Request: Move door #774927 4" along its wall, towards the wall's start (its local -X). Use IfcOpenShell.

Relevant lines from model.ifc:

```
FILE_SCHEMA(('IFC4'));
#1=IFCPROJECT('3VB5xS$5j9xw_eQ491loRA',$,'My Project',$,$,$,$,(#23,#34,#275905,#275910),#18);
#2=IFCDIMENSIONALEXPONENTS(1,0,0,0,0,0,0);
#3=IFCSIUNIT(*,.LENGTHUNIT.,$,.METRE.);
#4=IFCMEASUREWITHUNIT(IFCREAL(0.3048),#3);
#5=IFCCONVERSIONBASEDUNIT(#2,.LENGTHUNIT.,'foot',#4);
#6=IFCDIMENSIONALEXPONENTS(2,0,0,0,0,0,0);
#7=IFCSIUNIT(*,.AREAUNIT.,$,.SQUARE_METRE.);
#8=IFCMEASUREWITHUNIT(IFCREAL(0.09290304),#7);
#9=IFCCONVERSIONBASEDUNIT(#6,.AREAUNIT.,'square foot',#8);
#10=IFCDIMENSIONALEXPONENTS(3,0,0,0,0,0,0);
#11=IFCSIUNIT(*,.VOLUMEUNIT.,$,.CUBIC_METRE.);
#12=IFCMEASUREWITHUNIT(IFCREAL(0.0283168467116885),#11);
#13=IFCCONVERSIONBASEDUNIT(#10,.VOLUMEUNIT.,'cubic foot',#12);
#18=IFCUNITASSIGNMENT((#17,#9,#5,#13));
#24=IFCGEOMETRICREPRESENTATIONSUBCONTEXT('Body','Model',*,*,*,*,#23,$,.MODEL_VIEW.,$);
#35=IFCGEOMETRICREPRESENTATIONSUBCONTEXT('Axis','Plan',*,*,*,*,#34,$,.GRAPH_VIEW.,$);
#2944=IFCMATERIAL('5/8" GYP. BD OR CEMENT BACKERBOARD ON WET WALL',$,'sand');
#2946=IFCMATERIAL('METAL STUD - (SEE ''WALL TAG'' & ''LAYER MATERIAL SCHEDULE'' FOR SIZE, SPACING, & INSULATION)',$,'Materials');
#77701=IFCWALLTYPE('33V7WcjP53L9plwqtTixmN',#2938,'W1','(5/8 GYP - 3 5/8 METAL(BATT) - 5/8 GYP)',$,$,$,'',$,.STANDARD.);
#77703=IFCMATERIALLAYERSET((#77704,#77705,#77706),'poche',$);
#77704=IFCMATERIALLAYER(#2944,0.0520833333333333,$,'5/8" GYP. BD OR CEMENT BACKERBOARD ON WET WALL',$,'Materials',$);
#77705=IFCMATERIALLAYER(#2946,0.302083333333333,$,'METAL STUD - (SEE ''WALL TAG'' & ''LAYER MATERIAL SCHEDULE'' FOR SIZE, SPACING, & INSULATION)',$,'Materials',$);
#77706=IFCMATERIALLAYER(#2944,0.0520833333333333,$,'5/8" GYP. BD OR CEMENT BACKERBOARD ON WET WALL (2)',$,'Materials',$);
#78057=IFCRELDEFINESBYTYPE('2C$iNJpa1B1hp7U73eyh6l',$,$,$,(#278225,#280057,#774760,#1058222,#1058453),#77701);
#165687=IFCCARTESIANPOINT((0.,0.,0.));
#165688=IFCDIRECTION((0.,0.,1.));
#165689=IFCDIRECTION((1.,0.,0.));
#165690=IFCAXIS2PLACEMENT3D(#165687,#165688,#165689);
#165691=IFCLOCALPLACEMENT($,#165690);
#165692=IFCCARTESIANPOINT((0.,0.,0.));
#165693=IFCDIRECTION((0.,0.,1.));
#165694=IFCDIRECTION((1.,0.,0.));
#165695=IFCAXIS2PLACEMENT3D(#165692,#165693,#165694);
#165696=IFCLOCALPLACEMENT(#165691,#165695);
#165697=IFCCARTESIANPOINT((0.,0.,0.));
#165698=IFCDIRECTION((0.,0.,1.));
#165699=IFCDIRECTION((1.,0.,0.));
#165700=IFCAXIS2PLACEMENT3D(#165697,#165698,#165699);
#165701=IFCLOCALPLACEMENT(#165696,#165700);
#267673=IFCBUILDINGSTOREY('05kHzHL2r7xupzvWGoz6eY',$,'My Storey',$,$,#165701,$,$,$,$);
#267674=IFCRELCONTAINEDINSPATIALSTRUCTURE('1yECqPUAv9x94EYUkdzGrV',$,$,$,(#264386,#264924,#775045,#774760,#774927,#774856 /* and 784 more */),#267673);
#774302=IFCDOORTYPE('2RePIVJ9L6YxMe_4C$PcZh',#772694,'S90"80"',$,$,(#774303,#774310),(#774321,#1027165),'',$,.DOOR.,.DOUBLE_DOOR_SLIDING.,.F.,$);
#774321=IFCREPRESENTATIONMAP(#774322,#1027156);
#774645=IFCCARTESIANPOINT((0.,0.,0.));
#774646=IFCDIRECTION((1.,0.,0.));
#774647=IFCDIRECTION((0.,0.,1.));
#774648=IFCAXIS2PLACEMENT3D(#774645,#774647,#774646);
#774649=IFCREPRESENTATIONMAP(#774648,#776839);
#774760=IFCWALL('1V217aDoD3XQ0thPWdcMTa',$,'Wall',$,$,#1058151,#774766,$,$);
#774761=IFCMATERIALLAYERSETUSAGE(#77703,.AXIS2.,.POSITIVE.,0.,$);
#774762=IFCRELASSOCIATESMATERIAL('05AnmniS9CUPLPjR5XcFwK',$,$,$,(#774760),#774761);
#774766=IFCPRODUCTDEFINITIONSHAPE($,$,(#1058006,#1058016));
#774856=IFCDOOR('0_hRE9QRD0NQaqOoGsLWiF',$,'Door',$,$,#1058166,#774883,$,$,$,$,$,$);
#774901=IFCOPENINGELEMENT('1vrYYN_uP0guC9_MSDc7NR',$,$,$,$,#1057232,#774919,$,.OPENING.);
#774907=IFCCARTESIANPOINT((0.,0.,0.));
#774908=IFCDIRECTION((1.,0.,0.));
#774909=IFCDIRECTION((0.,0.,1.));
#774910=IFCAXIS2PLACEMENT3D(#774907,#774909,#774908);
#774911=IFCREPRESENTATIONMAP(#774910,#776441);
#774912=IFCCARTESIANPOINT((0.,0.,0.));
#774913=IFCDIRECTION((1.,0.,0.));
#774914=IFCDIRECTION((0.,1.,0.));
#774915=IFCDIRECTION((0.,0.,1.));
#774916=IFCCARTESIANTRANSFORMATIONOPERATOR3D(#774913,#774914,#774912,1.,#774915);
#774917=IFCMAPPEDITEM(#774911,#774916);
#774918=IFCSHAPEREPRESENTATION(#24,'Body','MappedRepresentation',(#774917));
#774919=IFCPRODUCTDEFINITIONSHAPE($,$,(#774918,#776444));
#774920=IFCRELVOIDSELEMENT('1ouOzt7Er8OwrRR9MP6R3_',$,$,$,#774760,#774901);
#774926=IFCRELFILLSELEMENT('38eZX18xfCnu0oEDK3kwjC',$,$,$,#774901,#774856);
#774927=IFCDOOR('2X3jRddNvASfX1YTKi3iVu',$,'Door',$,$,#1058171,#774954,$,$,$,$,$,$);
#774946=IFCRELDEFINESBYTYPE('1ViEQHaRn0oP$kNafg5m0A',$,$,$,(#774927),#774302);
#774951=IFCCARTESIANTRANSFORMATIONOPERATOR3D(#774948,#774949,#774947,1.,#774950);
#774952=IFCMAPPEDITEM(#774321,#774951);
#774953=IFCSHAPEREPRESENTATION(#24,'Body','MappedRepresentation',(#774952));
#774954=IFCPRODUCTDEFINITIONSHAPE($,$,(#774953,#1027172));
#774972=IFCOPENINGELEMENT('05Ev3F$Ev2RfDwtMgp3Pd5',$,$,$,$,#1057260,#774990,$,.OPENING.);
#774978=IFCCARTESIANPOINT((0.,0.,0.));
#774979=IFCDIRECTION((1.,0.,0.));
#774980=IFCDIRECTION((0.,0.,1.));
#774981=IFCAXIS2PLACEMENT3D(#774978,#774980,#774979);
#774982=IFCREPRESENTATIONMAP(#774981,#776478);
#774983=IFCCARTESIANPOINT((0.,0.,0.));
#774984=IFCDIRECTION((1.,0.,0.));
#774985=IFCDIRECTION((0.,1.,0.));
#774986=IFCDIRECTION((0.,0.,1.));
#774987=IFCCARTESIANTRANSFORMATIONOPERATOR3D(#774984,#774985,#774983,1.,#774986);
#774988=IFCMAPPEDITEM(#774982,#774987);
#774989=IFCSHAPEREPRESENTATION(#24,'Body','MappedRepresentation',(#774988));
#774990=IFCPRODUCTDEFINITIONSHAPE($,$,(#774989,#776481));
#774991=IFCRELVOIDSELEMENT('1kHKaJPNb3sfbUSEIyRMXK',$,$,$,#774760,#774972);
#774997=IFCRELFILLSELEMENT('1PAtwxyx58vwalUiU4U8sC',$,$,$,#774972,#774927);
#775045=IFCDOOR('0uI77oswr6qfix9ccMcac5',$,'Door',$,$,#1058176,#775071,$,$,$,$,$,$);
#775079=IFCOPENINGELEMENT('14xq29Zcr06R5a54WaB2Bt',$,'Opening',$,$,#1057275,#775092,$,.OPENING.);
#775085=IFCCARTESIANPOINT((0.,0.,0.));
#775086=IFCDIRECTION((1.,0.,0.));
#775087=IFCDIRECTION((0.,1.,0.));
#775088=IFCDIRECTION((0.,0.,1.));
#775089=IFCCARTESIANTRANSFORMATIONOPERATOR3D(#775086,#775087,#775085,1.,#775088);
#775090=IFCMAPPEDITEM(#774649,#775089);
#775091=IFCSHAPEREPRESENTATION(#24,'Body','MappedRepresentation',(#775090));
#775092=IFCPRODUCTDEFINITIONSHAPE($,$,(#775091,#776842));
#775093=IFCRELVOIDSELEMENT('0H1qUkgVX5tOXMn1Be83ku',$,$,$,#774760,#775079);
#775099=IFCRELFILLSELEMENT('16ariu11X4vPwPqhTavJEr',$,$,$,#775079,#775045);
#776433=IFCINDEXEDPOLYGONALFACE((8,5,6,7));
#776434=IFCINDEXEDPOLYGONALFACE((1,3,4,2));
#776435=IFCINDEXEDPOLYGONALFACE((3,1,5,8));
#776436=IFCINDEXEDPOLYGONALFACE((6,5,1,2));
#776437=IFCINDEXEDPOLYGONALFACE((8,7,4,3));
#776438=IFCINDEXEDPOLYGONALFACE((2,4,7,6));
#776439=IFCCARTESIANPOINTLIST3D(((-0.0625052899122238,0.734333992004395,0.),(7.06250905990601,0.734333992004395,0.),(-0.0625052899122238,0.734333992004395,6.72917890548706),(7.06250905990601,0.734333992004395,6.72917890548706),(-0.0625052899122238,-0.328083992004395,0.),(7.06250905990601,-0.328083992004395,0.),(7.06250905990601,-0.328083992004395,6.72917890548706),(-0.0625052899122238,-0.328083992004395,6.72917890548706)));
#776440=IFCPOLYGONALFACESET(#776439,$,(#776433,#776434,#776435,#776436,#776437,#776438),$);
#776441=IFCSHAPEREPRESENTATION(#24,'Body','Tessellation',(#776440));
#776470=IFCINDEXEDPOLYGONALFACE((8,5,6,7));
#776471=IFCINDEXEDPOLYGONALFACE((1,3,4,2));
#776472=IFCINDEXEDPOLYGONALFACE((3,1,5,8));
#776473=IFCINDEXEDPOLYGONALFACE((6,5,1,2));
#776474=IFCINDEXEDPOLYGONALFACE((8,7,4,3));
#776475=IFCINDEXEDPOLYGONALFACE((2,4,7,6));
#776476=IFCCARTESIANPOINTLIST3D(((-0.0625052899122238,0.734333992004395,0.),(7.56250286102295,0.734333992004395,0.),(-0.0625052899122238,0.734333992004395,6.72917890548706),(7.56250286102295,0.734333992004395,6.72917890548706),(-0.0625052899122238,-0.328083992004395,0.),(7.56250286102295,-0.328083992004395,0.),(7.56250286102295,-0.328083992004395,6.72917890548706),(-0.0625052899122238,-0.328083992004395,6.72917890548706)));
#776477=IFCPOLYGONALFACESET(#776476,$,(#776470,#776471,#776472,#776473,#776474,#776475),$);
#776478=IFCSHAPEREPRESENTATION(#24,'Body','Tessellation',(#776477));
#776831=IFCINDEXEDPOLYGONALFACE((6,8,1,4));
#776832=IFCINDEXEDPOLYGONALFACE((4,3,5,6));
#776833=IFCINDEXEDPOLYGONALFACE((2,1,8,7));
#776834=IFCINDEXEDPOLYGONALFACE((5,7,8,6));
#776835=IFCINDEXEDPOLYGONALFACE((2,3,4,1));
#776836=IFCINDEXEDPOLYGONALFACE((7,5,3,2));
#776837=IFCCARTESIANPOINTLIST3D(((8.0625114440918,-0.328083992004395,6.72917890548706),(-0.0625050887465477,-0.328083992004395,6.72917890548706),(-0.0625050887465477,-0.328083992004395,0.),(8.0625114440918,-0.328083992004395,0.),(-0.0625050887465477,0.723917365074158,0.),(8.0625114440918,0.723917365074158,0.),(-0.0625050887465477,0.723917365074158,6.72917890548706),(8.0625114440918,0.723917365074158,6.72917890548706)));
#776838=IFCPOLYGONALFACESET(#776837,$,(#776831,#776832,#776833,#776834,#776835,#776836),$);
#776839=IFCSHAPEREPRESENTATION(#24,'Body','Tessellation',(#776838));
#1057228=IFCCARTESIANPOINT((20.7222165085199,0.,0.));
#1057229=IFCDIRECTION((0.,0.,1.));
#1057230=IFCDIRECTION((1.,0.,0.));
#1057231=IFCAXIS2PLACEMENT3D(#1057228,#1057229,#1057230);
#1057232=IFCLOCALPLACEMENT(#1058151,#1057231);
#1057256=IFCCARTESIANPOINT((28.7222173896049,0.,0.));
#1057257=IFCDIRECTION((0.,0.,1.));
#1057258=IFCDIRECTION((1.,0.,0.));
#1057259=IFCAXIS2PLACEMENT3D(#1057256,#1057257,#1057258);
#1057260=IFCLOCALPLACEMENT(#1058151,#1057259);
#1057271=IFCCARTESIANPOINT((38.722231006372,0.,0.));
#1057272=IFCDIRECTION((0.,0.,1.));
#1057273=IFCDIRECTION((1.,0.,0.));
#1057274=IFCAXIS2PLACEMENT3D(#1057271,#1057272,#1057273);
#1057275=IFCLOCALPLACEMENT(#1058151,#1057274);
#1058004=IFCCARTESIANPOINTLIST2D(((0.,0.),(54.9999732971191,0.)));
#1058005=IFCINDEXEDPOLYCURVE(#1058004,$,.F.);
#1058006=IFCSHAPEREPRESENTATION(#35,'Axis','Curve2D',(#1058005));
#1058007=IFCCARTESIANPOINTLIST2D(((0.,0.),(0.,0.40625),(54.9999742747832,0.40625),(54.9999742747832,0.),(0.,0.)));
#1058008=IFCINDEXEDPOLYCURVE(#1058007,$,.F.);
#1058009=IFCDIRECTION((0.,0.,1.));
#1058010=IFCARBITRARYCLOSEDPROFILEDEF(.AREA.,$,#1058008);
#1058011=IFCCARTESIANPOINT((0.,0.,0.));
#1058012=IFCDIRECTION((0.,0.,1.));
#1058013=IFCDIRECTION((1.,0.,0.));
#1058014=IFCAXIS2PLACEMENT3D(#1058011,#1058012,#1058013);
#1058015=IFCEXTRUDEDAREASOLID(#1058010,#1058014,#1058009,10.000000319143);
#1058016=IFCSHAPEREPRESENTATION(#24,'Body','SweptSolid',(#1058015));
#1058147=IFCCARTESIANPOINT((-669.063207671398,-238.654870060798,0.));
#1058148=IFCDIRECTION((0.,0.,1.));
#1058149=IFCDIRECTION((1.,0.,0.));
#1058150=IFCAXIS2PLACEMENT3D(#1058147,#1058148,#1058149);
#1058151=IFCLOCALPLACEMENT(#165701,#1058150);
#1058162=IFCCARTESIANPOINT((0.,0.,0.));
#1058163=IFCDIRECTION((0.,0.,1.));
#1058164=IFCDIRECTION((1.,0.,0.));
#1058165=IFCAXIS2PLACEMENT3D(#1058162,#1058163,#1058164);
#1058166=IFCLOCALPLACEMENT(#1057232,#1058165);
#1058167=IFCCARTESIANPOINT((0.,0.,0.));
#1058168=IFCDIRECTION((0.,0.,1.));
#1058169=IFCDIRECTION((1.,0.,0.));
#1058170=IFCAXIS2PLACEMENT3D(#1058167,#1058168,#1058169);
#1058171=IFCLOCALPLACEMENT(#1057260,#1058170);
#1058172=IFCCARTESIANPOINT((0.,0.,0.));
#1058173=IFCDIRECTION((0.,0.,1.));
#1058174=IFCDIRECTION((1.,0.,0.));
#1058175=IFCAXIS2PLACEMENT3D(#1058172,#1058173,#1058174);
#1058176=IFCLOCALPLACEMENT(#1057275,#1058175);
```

```python
import ifcopenshell
import ifcopenshell.api.geometry
import ifcopenshell.util.placement
import ifcopenshell.util.unit

model = ifcopenshell.open("model.ifc")
unit_scale = ifcopenshell.util.unit.calculate_unit_scale(model)

door = model.by_id(774927)
opening = door.FillsVoids[0].RelatingOpeningElement
wall = opening.VoidsElements[0].RelatingBuildingElement

wall_matrix = ifcopenshell.util.placement.get_local_placement(wall.ObjectPlacement)
shift = wall_matrix[:3, 0] * -4 * 0.0254 / unit_scale
before = ifcopenshell.util.placement.get_local_placement(door.ObjectPlacement)[:3, 3].copy()

# The door is placed relative to its opening, so it follows when the opening moves.
matrix = ifcopenshell.util.placement.get_local_placement(opening.ObjectPlacement)
matrix[:3, 3] += shift
ifcopenshell.api.geometry.edit_object_placement(
    model, product=opening, matrix=matrix, is_si=False, should_transform_children=True
)

after = ifcopenshell.util.placement.get_local_placement(door.ObjectPlacement)[:3, 3]
print("door moved by", (after - before).round(3) + 0.0)

model.write("model_updated.ifc")
```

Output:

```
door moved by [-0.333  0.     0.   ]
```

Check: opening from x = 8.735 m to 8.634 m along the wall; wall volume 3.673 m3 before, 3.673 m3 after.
